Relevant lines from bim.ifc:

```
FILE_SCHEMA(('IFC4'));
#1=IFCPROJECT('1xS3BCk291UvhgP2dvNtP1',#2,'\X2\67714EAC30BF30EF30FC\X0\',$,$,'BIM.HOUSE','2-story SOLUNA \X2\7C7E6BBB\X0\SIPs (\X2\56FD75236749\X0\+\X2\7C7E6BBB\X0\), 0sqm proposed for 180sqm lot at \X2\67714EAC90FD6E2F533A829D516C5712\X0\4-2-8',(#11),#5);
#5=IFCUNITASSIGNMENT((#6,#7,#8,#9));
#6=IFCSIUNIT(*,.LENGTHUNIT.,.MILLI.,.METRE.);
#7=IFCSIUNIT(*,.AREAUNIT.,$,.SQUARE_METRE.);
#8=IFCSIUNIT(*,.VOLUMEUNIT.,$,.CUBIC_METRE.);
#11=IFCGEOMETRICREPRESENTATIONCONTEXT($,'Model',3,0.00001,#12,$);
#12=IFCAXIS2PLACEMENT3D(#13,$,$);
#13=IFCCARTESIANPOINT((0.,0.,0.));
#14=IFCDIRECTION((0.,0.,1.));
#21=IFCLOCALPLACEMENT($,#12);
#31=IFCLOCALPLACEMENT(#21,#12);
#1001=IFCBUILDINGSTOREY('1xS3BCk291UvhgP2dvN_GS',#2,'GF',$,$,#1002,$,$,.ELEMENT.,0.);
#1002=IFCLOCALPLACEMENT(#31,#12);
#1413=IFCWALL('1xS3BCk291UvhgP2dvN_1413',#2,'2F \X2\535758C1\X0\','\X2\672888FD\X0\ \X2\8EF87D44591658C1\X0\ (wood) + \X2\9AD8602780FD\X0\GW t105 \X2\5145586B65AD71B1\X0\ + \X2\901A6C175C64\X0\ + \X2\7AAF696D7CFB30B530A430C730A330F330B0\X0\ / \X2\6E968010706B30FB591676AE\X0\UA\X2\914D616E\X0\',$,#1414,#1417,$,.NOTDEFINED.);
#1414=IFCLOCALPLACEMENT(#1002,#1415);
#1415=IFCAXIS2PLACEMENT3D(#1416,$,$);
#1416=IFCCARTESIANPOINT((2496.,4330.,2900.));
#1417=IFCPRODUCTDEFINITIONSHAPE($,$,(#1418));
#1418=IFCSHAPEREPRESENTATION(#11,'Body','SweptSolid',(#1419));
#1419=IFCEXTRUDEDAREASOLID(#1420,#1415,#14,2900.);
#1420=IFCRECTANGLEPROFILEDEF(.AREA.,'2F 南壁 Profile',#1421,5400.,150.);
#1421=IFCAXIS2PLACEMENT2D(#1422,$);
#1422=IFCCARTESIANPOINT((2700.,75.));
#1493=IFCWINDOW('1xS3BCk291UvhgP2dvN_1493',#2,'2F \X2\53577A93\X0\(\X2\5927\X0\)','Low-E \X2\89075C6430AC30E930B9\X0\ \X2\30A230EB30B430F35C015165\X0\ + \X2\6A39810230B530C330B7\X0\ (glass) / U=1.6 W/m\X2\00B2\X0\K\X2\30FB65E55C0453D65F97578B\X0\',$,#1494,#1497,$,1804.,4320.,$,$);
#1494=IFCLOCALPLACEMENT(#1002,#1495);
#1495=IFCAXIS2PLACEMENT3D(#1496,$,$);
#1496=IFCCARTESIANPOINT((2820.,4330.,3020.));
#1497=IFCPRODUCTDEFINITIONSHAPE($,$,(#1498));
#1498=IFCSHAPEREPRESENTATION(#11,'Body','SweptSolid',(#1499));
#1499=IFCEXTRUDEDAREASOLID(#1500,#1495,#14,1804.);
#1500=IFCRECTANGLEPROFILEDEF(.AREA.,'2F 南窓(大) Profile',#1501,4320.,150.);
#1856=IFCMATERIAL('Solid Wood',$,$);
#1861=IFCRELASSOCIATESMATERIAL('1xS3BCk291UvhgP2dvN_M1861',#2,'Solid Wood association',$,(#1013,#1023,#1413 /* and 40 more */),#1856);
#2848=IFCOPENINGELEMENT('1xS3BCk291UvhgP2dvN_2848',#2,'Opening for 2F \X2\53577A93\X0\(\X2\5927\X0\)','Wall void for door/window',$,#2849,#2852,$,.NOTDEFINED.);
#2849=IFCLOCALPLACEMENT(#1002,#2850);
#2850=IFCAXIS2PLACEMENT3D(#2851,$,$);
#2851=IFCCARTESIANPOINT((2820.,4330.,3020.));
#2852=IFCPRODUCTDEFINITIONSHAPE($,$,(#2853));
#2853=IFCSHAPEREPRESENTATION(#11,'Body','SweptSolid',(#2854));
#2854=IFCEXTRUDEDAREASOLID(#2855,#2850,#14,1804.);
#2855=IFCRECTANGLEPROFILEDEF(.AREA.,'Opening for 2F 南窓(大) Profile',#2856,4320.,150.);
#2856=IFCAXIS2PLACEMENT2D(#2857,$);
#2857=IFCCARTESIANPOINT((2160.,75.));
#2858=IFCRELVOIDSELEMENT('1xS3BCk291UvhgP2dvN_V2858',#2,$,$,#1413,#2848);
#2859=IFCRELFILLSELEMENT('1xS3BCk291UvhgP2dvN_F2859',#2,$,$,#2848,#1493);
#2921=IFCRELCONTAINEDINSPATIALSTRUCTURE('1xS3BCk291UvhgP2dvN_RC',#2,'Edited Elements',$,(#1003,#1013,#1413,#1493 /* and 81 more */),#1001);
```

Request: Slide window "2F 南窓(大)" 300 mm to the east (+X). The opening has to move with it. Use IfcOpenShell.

```python
import ifcopenshell
import ifcopenshell.api.geometry
import ifcopenshell.util.placement
import ifcopenshell.util.unit

model = ifcopenshell.open("bim.ifc")
unit_scale = ifcopenshell.util.unit.calculate_unit_scale(model)

window = model.by_guid("1xS3BCk291UvhgP2dvN_1493")
opening = window.FillsVoids[0].RelatingOpeningElement
wall = opening.VoidsElements[0].RelatingBuildingElement

wall_matrix = ifcopenshell.util.placement.get_local_placement(wall.ObjectPlacement)
shift = wall_matrix[:3, 0] * 0.3 / unit_scale
before = ifcopenshell.util.placement.get_local_placement(window.ObjectPlacement)[:3, 3].copy()

# The window is not placed relative to its opening, so move both.
for product in (opening, window):
    matrix = ifcopenshell.util.placement.get_local_placement(product.ObjectPlacement)
    matrix[:3, 3] += shift
    ifcopenshell.api.geometry.edit_object_placement(model, product=product, matrix=matrix, is_si=False)

after = ifcopenshell.util.placement.get_local_placement(window.ObjectPlacement)[:3, 3]
print("window moved by", (after - before).round(3) + 0.0)

model.write("bim_updated.ifc")
```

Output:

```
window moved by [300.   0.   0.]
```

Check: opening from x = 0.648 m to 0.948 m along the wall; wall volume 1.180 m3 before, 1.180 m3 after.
